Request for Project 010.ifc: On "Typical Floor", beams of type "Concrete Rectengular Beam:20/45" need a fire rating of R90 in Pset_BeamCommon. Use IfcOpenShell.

First a look at what the model holds.

```python
import ifcopenshell
import ifcopenshell.util.element

model = ifcopenshell.open("Project 010.ifc")
print(model.schema)
storey = next(s for s in model.by_type("IfcBuildingStorey") if s.Name == "Typical Floor")
beams = [e for e in ifcopenshell.util.element.get_decomposition(storey) if e.is_a("IfcBeam")]
seen = {}
for e in beams:
    element_type = ifcopenshell.util.element.get_type(e)
    key = (element_type.Name if element_type != e and element_type else None, ifcopenshell.util.element.get_pset(e, "Pset_BeamCommon", "FireRating"))
    seen[key] = seen.get(key, 0) + 1
for (name, value), count in sorted(seen.items(), key=str):
    print(count, "x", name, "|", value)
```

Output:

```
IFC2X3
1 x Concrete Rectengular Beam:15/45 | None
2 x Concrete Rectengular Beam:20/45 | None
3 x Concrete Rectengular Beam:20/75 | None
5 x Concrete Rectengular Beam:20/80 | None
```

```python
import ifcopenshell
import ifcopenshell.api.pset
import ifcopenshell.util.element

model = ifcopenshell.open("Project 010.ifc")

storey = next(s for s in model.by_type("IfcBuildingStorey") if s.Name == "Typical Floor")
beams = [e for e in ifcopenshell.util.element.get_decomposition(storey) if e.is_a("IfcBeam")]

count = 0
for e in beams:
    element_type = ifcopenshell.util.element.get_type(e)
    if element_type in (None, e) or element_type.Name != "Concrete Rectengular Beam:20/45":
        continue
    # add_pset returns the element's existing set when there is one.
    pset = ifcopenshell.api.pset.add_pset(model, product=e, name="Pset_BeamCommon")
    ifcopenshell.api.pset.edit_pset(model, pset=pset, properties={"FireRating": "R90"})
    count += 1

print(count, "beams updated")

model.write("Project 010_updated.ifc")
```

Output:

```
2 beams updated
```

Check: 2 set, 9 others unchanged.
